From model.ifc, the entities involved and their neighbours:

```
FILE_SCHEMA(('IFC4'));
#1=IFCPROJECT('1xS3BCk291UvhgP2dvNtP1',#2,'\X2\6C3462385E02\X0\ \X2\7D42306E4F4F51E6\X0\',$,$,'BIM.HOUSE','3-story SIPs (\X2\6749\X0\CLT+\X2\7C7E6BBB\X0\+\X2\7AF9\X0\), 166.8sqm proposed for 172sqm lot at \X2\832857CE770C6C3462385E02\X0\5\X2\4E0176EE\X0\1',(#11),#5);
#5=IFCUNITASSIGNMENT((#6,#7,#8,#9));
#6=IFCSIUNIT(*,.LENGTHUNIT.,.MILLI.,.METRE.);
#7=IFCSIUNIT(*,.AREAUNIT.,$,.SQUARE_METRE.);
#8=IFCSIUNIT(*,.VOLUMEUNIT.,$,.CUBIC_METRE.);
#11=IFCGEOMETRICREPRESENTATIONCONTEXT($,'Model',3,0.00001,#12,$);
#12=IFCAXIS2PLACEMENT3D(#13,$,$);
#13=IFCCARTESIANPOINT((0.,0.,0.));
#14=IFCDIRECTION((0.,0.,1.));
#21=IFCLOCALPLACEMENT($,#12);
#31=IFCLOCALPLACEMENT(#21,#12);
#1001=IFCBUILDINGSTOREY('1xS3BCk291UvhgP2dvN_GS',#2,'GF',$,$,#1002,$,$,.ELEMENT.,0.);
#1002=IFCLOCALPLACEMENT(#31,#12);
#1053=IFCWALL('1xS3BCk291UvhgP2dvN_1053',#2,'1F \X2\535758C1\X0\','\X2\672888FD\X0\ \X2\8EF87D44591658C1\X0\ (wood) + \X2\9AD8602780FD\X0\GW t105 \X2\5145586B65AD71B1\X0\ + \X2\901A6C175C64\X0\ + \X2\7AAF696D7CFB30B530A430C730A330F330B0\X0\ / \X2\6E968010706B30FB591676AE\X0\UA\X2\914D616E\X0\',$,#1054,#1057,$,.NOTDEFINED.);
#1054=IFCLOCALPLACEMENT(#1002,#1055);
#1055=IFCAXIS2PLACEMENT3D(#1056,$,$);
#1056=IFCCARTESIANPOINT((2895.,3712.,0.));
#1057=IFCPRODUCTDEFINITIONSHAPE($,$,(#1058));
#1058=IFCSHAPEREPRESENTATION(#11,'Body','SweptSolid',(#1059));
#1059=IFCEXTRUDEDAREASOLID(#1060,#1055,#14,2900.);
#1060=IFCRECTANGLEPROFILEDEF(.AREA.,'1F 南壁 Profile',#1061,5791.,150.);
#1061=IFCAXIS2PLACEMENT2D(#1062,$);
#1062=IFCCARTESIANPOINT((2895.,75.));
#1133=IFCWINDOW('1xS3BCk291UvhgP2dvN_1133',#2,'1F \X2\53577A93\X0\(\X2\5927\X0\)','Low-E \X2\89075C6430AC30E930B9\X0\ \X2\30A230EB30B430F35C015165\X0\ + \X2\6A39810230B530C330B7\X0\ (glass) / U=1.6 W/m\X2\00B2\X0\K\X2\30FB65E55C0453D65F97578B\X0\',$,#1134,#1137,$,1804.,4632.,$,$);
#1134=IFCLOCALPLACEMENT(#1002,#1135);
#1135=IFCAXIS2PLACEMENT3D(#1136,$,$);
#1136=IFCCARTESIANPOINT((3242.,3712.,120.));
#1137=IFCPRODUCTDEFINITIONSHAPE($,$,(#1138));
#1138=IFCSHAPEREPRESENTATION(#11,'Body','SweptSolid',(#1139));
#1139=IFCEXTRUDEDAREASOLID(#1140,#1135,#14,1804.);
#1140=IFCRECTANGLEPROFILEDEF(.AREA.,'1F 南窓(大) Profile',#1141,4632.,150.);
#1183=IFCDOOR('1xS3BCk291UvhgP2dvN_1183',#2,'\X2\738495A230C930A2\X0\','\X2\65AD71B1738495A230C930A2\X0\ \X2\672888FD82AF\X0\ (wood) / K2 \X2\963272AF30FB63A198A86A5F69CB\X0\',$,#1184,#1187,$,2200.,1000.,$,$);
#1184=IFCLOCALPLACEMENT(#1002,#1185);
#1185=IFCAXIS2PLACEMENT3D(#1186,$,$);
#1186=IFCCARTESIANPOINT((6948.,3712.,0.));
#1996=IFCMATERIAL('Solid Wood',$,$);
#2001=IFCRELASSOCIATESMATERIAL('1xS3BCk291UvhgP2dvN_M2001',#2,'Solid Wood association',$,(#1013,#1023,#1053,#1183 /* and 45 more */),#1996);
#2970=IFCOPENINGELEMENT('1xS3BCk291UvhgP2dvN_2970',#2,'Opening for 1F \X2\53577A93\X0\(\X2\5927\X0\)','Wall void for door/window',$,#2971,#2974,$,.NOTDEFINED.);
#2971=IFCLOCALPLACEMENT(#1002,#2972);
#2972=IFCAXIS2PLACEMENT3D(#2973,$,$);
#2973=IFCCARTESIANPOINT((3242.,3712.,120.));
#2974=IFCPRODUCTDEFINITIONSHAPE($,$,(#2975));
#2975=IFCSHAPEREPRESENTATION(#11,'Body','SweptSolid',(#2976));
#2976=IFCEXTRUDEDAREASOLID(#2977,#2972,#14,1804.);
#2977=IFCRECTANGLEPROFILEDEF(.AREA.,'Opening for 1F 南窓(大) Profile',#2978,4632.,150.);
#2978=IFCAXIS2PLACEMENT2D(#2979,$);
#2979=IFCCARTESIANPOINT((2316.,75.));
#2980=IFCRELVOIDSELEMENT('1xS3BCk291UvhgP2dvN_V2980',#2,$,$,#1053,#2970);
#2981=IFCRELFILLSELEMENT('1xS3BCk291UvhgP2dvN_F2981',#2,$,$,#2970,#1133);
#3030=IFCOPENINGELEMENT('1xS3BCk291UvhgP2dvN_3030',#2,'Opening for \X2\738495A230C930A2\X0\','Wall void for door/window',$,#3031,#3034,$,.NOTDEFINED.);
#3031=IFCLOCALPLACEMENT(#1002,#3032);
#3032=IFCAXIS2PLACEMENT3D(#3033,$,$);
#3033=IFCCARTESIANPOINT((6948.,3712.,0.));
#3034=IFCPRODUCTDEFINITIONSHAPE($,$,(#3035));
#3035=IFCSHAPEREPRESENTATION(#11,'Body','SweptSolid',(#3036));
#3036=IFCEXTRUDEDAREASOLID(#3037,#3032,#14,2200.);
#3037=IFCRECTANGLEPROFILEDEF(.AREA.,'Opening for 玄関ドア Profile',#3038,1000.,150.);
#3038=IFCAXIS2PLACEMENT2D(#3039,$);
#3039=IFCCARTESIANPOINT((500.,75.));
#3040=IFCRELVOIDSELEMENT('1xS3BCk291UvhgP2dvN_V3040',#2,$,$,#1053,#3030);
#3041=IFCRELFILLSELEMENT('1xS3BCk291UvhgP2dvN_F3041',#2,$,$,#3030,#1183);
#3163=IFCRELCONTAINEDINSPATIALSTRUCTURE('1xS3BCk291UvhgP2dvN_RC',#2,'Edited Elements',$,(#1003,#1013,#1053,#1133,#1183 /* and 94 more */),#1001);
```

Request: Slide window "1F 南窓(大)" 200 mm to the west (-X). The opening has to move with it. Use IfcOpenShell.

```python
import ifcopenshell
import ifcopenshell.api.geometry
import ifcopenshell.util.placement
import ifcopenshell.util.unit

model = ifcopenshell.open("model.ifc")
unit_scale = ifcopenshell.util.unit.calculate_unit_scale(model)

window = model.by_id(1133)
opening = window.FillsVoids[0].RelatingOpeningElement
wall = opening.VoidsElements[0].RelatingBuildingElement

wall_matrix = ifcopenshell.util.placement.get_local_placement(wall.ObjectPlacement)
shift = wall_matrix[:3, 0] * -0.2 / unit_scale
before = ifcopenshell.util.placement.get_local_placement(window.ObjectPlacement)[:3, 3].copy()

# The window is not placed relative to its opening, so move both.
for product in (opening, window):
    matrix = ifcopenshell.util.placement.get_local_placement(product.ObjectPlacement)
    matrix[:3, 3] += shift
    ifcopenshell.api.geometry.edit_object_placement(model, product=product, matrix=matrix, is_si=False)

after = ifcopenshell.util.placement.get_local_placement(window.ObjectPlacement)[:3, 3]
print("window moved by", (after - before).round(3) + 0.0)

model.write("model_v2.ifc")
```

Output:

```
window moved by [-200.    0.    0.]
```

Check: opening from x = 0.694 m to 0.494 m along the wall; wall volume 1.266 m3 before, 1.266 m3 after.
